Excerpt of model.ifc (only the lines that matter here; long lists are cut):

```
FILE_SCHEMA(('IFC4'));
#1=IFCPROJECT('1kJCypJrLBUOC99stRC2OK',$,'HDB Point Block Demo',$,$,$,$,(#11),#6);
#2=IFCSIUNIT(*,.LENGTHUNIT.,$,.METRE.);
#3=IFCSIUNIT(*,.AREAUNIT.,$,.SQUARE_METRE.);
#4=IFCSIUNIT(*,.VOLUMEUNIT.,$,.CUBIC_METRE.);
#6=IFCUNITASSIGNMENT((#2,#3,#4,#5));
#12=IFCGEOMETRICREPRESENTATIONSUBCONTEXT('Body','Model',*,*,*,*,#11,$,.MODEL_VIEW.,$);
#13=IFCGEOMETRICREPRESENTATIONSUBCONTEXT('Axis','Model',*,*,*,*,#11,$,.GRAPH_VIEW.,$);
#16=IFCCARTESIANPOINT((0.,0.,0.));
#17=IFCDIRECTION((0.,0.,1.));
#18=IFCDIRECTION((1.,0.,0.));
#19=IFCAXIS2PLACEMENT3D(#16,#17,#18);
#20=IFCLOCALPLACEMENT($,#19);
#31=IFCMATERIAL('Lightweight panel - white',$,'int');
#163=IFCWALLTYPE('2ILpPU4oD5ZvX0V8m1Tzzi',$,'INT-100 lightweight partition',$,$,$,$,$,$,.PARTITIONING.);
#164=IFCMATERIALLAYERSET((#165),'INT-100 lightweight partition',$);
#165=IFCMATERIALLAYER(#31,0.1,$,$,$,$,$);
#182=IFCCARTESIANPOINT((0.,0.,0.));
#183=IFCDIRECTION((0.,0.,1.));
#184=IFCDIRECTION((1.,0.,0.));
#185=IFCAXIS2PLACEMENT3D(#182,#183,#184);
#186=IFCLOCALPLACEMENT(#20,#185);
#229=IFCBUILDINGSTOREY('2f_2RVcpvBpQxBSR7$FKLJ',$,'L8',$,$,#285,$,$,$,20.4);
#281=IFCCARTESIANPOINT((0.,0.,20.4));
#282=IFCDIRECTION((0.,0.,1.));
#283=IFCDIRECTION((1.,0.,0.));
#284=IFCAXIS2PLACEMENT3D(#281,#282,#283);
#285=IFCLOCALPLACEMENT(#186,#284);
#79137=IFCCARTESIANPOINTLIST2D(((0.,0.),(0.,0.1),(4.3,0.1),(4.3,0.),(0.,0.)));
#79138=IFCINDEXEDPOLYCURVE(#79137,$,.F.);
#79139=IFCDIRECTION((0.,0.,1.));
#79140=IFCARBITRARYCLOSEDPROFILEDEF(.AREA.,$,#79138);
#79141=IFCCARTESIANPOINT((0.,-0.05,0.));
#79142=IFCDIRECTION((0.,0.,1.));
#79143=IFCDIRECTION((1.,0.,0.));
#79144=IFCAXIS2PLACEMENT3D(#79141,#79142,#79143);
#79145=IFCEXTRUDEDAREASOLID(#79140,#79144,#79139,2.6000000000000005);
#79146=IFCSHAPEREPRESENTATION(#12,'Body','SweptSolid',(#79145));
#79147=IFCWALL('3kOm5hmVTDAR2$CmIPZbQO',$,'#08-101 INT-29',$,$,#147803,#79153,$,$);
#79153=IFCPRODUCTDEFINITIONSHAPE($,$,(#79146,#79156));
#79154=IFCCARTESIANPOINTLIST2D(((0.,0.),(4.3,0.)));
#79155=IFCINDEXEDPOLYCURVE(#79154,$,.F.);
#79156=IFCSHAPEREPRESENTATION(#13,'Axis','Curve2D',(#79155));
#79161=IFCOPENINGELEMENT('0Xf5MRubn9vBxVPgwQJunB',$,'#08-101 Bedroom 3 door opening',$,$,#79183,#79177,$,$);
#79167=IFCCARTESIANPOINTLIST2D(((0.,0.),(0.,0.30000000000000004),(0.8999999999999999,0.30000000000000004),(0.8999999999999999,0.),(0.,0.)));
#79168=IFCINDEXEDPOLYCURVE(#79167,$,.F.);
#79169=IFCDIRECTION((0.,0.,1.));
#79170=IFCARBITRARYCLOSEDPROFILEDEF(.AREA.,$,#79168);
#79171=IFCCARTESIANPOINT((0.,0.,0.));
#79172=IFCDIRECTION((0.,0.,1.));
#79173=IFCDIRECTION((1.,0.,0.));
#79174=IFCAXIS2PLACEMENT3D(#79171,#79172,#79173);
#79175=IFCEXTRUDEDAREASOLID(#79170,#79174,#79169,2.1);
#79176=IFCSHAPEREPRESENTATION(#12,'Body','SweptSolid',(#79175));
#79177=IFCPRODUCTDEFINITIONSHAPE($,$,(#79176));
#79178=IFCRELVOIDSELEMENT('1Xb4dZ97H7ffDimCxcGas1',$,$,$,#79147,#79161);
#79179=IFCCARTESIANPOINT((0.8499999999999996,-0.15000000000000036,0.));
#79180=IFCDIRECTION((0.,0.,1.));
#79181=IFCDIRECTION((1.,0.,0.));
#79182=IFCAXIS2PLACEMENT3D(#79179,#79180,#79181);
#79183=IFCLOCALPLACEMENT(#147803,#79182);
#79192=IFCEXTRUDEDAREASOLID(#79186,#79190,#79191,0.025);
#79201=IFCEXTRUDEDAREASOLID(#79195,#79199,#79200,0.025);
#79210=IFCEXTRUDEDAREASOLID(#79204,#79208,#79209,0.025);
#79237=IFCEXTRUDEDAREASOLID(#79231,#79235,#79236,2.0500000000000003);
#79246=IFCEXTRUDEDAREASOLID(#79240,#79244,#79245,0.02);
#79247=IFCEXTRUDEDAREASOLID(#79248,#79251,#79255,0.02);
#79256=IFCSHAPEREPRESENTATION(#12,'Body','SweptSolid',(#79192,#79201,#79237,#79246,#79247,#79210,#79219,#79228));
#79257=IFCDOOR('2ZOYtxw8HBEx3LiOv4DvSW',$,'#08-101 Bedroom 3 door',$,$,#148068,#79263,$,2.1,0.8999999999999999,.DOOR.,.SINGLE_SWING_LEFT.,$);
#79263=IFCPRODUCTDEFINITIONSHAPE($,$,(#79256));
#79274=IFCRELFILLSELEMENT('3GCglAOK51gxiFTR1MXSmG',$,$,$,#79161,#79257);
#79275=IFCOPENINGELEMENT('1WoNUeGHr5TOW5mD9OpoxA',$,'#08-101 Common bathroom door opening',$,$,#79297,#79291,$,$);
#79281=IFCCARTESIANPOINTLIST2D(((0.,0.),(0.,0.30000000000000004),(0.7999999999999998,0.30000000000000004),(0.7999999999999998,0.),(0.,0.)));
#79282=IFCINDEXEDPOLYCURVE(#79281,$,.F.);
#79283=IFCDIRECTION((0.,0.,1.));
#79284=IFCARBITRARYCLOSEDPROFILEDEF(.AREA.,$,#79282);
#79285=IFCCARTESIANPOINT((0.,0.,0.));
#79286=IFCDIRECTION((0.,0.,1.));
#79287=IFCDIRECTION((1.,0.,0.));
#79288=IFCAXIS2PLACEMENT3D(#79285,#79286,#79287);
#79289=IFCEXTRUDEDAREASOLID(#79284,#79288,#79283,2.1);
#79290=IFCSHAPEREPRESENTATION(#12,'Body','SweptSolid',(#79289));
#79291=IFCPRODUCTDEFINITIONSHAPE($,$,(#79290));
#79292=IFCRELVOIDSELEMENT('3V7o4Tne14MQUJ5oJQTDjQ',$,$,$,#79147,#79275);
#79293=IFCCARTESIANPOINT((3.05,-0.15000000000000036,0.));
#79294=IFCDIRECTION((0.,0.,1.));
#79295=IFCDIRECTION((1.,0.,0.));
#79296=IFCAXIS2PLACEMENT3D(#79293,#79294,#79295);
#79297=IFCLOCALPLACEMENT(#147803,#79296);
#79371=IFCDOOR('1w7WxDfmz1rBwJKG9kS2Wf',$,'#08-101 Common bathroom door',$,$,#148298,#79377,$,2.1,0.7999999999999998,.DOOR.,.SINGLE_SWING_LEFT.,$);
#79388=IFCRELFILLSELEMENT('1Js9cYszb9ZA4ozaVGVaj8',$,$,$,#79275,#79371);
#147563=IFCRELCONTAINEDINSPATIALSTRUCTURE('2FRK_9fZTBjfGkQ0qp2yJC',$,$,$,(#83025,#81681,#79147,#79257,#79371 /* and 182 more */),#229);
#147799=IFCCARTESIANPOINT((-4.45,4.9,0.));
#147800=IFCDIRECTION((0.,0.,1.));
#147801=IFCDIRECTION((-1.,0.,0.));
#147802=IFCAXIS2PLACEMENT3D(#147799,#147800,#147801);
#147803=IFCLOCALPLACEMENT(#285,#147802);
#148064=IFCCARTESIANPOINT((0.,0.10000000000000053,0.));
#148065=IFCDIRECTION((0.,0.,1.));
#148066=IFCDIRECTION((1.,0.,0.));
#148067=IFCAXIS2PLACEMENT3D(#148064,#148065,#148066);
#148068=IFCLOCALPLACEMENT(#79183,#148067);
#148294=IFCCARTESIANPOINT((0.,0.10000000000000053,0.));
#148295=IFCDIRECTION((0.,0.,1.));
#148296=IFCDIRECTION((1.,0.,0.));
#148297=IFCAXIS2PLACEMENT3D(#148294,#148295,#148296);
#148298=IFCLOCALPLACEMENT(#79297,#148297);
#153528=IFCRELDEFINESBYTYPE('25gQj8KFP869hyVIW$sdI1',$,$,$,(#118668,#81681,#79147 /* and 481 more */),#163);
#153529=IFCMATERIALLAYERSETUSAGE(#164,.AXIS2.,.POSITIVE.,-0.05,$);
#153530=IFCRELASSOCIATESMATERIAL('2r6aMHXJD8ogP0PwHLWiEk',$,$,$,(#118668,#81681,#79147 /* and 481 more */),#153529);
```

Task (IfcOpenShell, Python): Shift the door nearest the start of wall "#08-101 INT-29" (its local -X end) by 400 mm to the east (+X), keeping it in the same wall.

```python
import ifcopenshell
import ifcopenshell.api.geometry
import ifcopenshell.util.placement
import ifcopenshell.util.unit

model = ifcopenshell.open("model.ifc")
unit_scale = ifcopenshell.util.unit.calculate_unit_scale(model)

door = model.by_guid("2ZOYtxw8HBEx3LiOv4DvSW")
opening = door.FillsVoids[0].RelatingOpeningElement
wall = opening.VoidsElements[0].RelatingBuildingElement

wall_matrix = ifcopenshell.util.placement.get_local_placement(wall.ObjectPlacement)
shift = wall_matrix[:3, 0] * -0.4 / unit_scale
before = ifcopenshell.util.placement.get_local_placement(door.ObjectPlacement)[:3, 3].copy()

# The door is placed relative to its opening, so it follows when the opening moves.
matrix = ifcopenshell.util.placement.get_local_placement(opening.ObjectPlacement)
matrix[:3, 3] += shift
ifcopenshell.api.geometry.edit_object_placement(
    model, product=opening, matrix=matrix, is_si=False, should_transform_children=True
)

after = ifcopenshell.util.placement.get_local_placement(door.ObjectPlacement)[:3, 3]
print("door moved by", (after - before).round(3) + 0.0)

model.write("model_v2.ifc")
```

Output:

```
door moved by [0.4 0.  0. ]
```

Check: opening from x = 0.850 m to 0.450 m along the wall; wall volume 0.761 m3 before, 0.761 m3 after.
